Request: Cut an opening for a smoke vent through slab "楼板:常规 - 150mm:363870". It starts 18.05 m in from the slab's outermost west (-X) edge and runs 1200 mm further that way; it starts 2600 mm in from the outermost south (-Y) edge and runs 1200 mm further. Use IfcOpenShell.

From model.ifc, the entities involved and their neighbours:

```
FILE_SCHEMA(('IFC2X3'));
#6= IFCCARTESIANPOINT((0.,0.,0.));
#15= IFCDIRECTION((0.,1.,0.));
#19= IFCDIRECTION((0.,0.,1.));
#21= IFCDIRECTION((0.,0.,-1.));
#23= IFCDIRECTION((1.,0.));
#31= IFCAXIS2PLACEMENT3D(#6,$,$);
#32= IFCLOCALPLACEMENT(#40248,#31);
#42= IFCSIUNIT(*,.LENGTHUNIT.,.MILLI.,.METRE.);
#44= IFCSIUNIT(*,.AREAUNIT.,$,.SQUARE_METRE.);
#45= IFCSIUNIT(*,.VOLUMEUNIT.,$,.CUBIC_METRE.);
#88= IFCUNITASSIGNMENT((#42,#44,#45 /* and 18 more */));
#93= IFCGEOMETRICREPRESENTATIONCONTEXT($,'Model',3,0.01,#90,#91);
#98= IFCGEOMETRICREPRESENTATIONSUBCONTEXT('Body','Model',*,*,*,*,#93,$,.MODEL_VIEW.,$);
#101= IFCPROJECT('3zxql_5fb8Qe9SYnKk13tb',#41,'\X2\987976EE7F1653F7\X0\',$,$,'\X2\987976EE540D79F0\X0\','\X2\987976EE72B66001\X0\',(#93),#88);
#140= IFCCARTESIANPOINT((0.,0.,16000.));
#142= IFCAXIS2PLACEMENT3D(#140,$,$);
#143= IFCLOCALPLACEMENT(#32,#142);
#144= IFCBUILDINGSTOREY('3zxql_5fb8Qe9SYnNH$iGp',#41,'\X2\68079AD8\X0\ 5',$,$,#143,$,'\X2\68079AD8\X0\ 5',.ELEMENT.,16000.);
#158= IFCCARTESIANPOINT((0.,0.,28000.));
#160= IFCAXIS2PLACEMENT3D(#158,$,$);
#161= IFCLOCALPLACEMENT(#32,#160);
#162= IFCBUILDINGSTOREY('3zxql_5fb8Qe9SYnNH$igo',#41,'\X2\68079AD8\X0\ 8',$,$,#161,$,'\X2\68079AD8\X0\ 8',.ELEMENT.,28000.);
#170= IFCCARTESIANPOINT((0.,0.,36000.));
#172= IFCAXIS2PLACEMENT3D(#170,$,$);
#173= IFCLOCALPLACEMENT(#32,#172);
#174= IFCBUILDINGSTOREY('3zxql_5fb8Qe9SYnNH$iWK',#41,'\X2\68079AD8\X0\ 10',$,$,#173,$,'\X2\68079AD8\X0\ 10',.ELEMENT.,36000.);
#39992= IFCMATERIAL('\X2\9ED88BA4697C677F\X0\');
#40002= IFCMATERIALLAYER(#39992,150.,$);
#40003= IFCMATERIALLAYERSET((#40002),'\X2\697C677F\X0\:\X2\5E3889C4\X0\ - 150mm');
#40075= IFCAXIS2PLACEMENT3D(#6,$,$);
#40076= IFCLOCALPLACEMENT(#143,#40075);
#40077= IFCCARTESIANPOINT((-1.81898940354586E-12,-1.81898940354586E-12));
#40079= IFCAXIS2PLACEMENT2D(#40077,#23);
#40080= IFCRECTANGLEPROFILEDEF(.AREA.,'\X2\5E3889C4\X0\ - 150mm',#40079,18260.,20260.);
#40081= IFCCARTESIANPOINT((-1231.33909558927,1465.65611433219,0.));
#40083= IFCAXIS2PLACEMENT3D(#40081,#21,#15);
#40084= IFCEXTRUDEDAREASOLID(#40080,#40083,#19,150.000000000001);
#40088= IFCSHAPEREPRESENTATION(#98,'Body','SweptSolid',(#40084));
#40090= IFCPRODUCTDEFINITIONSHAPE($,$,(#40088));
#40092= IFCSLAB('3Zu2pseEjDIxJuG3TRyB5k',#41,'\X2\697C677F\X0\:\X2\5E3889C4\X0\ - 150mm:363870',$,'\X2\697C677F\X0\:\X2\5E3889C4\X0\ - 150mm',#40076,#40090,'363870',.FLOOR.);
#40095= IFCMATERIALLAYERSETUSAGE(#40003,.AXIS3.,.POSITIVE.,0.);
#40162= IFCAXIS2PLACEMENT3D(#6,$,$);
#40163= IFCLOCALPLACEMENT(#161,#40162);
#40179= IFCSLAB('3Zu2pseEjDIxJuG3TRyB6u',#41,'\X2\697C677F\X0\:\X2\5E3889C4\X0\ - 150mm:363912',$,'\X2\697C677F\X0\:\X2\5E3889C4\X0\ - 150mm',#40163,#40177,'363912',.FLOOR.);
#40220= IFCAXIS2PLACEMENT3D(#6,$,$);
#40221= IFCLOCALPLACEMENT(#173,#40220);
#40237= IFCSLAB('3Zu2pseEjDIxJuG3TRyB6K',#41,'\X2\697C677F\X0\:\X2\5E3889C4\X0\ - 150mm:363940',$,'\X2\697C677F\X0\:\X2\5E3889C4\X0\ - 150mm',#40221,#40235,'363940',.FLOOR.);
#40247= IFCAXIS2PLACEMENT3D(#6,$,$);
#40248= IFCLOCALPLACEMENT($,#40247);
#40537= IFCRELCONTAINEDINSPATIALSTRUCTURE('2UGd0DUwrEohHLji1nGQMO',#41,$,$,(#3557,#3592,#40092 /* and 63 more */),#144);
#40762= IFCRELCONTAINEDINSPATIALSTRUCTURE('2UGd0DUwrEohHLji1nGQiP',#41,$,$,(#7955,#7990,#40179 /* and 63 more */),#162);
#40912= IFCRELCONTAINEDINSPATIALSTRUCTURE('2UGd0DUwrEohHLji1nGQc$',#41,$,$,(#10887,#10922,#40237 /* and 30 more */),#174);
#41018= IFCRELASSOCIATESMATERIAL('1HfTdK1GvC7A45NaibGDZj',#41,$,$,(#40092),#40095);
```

```python
import numpy as np
import ifcopenshell
import ifcopenshell.api.feature
import ifcopenshell.api.geometry
import ifcopenshell.api.root
import ifcopenshell.geom
import ifcopenshell.util.placement
import ifcopenshell.util.representation
import ifcopenshell.util.shape
import ifcopenshell.util.unit

model = ifcopenshell.open("model.ifc")
unit_scale = ifcopenshell.util.unit.calculate_unit_scale(model)
settings = ifcopenshell.geom.settings()


def volume(element):
    """Net volume in cubic metres, openings subtracted."""
    shape = ifcopenshell.geom.create_shape(settings, element)
    return ifcopenshell.util.shape.get_volume(shape.geometry)


slab = model.by_guid("3Zu2pseEjDIxJuG3TRyB5k")
before = volume(slab)

# Extent in the slab's own axes, in metres. The edges named are its -X and -Y sides.
slab_shape = ifcopenshell.geom.create_shape(settings, slab)
vertices = ifcopenshell.util.shape.get_vertices(slab_shape.geometry)
x_min, y_min, bottom = vertices.min(axis=0)
top = vertices[:, 2].max()

opening = ifcopenshell.api.root.create_entity(model, ifc_class="IfcOpeningElement", name="Smoke vent opening")
context = ifcopenshell.util.representation.get_context(model, "Model", "Body", "MODEL_VIEW")
width, depth = 1.2, 1.2
outline = [(0.0, 0.0), (width, 0.0), (width, depth), (0.0, depth), (0.0, 0.0)]
# Overshoot both faces by 50 mm so the cut is clean.
shape = ifcopenshell.api.geometry.add_slab_representation(
    model, context=context, depth=top - bottom + 0.1, polyline=outline
)
ifcopenshell.api.geometry.assign_representation(model, product=opening, representation=shape)

matrix = ifcopenshell.util.placement.get_local_placement(slab.ObjectPlacement)
matrix[:, 3] = matrix @ np.append(np.array([x_min + 18.05, y_min + 2.6, bottom - 0.05]) / unit_scale, 1.0)
ifcopenshell.api.geometry.edit_object_placement(model, product=opening, matrix=matrix, is_si=False)
ifcopenshell.api.feature.add_feature(model, feature=opening, element=slab)

after = volume(slab)

print(f"slab volume {before:.3f} -> {after:.3f} m3")

model.write("model_edited.ifc")
```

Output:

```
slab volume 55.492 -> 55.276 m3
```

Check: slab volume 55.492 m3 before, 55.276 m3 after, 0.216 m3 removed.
